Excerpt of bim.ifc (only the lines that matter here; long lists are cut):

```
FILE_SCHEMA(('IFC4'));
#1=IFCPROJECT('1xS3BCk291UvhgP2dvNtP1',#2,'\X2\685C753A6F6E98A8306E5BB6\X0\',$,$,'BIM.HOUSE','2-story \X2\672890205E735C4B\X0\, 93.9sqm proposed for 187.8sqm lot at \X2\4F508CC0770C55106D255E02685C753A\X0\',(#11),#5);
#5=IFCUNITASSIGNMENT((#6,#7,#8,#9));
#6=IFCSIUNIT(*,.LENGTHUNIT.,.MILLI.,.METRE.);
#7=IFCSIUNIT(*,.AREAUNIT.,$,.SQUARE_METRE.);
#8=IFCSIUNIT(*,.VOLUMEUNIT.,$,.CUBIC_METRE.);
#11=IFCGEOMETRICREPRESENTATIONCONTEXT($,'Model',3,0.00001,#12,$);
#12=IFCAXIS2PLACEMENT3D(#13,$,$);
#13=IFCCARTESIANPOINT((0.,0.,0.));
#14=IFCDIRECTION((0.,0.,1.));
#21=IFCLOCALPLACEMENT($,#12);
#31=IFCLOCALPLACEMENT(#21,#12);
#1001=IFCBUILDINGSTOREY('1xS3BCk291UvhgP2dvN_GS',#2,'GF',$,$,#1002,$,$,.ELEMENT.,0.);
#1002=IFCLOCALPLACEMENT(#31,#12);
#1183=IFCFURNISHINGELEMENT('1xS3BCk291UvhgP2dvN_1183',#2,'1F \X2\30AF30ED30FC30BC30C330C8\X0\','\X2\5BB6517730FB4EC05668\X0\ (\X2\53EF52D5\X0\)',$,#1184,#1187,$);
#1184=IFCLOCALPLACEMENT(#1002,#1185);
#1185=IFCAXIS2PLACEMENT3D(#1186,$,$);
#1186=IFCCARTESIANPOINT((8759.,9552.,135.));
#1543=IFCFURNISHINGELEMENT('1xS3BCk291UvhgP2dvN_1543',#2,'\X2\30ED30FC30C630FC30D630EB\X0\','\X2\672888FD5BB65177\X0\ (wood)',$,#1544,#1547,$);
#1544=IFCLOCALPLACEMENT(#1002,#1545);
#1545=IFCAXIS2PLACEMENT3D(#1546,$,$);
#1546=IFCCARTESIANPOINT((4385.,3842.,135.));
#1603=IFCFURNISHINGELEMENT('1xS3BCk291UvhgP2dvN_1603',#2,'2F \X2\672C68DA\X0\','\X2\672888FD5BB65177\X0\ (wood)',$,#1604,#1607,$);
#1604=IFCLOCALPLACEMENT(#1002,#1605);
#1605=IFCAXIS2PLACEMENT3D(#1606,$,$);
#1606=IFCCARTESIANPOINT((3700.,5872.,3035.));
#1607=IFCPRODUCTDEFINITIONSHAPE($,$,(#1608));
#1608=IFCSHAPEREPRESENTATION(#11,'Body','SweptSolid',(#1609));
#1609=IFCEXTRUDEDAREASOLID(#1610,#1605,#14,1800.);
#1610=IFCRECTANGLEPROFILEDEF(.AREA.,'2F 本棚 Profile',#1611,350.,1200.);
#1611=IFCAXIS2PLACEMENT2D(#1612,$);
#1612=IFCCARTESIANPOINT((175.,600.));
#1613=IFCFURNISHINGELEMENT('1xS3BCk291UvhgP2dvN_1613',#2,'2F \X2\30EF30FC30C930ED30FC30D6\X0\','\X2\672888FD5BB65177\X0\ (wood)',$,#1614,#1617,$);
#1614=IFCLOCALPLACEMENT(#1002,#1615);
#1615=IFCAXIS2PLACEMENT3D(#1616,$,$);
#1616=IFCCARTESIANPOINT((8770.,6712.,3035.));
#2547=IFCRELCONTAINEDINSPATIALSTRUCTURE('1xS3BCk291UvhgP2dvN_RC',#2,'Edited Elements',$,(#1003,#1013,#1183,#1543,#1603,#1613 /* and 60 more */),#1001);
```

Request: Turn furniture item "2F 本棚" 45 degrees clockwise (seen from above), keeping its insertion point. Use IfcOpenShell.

```python
import ifcopenshell
import ifcopenshell.api.geometry
import ifcopenshell.util.placement

model = ifcopenshell.open("bim.ifc")

item = model.by_id(1603)
matrix = ifcopenshell.util.placement.get_local_placement(item.ObjectPlacement)
matrix = matrix @ ifcopenshell.util.placement.rotation(-45, "Z")
ifcopenshell.api.geometry.edit_object_placement(model, product=item, matrix=matrix, is_si=False)

print(ifcopenshell.util.placement.get_local_placement(item.ObjectPlacement).round(3) + 0.0)

model.write("bim_v2.ifc")
```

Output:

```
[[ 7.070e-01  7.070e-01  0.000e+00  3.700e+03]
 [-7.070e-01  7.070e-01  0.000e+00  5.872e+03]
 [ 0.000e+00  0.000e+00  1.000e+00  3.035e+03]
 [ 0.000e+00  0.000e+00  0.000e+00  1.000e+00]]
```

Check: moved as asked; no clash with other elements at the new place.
